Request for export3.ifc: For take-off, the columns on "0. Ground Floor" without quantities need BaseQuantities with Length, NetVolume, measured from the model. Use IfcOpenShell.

First a look at what the model holds.

```python
import ifcopenshell
import ifcopenshell.util.element
import ifcopenshell.util.unit

model = ifcopenshell.open("export3.ifc")
print(model.schema)
for unit_type in ("LENGTHUNIT", "AREAUNIT", "VOLUMEUNIT"):
    print(unit_type, ifcopenshell.util.unit.calculate_unit_scale(model, unit_type))
storey = next(s for s in model.by_type("IfcBuildingStorey") if s.Name == "0. Ground Floor")
columns = [e for e in ifcopenshell.util.element.get_decomposition(storey) if e.is_a("IfcColumn")]
for e in sorted(columns, key=lambda e: e.id()):
    print(e.id(), e.is_a(), e.Name, list(ifcopenshell.util.element.get_psets(e, qtos_only=True)), sep=" | ")
```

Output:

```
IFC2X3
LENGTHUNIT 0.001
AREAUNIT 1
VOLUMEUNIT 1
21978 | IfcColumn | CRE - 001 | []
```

```python
import ifcopenshell
import ifcopenshell.api.pset
import ifcopenshell.geom
import ifcopenshell.util.element
import ifcopenshell.util.shape
import ifcopenshell.util.unit

model = ifcopenshell.open("export3.ifc")
unit_scale = ifcopenshell.util.unit.calculate_unit_scale(model)
volume_scale = ifcopenshell.util.unit.calculate_unit_scale(model, "VOLUMEUNIT")
settings = ifcopenshell.geom.settings()

storey = next(s for s in model.by_type("IfcBuildingStorey") if s.Name == "0. Ground Floor")
columns = [e for e in ifcopenshell.util.element.get_decomposition(storey) if e.is_a("IfcColumn")]

for e in sorted(columns, key=lambda e: e.id()):
    if ifcopenshell.util.element.get_psets(e, qtos_only=True, should_inherit=False):
        continue
    # Geometry comes back in metres, in the element's own axes.
    shape = ifcopenshell.geom.create_shape(settings, e)
    values = {
        "Length": ifcopenshell.util.shape.get_z(shape.geometry) / unit_scale,
        "NetVolume": ifcopenshell.util.shape.get_volume(shape.geometry) / volume_scale,
    }
    qto = ifcopenshell.api.pset.add_qto(model, product=e, name="BaseQuantities")
    ifcopenshell.api.pset.edit_qto(model, qto=qto, properties=values)
    print(e.id(), {k: round(v, 3) for k, v in values.items()})

model.write("export3_updated.ifc")
```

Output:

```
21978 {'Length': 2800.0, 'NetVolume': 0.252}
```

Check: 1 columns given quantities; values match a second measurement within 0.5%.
